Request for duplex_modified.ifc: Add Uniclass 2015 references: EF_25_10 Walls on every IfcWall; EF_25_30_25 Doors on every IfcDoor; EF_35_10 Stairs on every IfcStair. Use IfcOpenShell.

First a look at what the model holds.

```python
import ifcopenshell

model = ifcopenshell.open("duplex_modified.ifc")
print(model.schema)
print("classifications:", [c.Name for c in model.by_type("IfcClassification")])
for ifc_class in ("IfcDoor", "IfcRoof", "IfcStair", "IfcWall", "IfcWindow"):
    print(ifc_class, len(model.by_type(ifc_class)))
```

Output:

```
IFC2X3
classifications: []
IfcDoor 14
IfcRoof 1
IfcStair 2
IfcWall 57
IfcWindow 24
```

```python
import ifcopenshell
import ifcopenshell.api.classification

model = ifcopenshell.open("duplex_modified.ifc")

# IFC2X3 requires Source and Edition and has no link from the project to the system.
system = model.create_entity("IfcClassification", Source="NBS", Edition="2015", Name="Uniclass 2015")

codes = {
    "IfcWall": ("EF_25_10", "Walls"),
    "IfcDoor": ("EF_25_30_25", "Doors"),
    "IfcStair": ("EF_35_10", "Stairs"),
}
for ifc_class, (code, name) in codes.items():
    products = model.by_type(ifc_class)
    ifcopenshell.api.classification.add_reference(
        model, products=products, classification=system, identification=code, name=name
    )
    print(code, len(products))

model.write("duplex_modified_updated.ifc")
```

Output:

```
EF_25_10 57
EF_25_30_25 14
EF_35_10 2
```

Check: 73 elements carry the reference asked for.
